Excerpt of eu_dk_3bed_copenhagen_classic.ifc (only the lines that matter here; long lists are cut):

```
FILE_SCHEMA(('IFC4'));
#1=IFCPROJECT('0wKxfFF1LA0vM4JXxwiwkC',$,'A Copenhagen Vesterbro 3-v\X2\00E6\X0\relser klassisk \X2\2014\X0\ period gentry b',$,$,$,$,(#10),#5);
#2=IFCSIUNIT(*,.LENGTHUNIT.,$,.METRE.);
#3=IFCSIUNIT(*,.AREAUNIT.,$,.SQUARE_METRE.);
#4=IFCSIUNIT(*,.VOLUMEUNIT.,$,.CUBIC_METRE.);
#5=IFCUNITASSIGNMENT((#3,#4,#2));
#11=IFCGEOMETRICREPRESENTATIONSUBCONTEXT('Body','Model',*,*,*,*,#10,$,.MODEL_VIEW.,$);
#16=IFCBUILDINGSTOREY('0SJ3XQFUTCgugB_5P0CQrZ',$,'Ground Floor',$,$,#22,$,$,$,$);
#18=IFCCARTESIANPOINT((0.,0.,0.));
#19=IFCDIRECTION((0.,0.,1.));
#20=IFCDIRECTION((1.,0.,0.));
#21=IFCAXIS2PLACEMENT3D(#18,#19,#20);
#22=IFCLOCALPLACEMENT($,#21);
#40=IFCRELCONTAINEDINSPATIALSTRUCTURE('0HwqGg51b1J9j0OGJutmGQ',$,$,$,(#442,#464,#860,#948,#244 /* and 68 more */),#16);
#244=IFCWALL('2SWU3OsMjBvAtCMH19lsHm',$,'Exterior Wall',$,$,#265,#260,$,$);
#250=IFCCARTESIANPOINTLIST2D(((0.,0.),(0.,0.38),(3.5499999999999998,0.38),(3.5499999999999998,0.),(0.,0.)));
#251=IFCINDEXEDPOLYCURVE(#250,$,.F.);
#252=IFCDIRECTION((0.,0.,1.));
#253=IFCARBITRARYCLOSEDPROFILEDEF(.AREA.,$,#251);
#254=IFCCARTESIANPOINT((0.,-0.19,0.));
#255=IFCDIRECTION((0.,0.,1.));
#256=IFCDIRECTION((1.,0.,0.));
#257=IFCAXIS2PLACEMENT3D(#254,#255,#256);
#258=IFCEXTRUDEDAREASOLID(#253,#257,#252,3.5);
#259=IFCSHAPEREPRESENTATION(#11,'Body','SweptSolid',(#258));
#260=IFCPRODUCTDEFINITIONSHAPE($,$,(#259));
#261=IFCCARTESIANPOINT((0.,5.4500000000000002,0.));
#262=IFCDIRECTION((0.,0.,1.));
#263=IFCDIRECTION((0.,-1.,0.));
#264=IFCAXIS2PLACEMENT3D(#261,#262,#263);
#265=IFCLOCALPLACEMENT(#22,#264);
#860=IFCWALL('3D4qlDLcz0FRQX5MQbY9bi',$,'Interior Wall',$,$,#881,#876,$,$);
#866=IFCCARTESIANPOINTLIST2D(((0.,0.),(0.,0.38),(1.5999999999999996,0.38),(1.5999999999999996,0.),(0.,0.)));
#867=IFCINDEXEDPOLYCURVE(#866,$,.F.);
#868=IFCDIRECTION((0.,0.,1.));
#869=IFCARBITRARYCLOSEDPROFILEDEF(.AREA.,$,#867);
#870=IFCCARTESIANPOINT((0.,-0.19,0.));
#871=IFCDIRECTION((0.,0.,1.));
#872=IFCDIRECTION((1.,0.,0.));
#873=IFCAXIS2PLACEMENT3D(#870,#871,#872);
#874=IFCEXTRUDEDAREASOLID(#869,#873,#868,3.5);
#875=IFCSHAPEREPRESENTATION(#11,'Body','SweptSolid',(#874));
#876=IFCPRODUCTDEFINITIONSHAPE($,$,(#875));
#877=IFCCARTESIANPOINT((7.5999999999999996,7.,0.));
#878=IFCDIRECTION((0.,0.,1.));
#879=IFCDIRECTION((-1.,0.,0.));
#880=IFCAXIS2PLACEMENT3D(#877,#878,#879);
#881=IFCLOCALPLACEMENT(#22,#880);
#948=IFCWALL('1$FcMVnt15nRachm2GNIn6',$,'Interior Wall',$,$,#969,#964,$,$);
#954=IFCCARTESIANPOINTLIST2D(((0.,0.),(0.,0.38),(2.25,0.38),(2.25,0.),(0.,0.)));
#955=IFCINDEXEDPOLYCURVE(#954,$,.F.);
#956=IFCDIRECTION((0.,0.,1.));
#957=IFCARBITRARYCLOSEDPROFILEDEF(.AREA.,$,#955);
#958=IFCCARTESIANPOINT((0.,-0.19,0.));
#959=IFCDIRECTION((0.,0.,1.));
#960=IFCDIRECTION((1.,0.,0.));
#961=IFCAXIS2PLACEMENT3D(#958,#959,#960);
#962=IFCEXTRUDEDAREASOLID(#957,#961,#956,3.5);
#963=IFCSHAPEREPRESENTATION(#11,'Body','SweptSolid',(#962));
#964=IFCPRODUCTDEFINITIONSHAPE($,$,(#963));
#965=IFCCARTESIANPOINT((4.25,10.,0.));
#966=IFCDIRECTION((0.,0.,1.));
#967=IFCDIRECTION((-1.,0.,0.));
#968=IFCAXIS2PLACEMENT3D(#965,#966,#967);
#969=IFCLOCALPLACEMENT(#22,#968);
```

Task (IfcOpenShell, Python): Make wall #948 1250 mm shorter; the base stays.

```python
import ifcopenshell
import ifcopenshell.geom
import ifcopenshell.util.representation
import ifcopenshell.util.shape
import ifcopenshell.util.unit

model = ifcopenshell.open("eu_dk_3bed_copenhagen_classic.ifc")
unit_scale = ifcopenshell.util.unit.calculate_unit_scale(model)
settings = ifcopenshell.geom.settings()


def volume(element):
    """Net volume in cubic metres, openings subtracted."""
    shape = ifcopenshell.geom.create_shape(settings, element)
    return ifcopenshell.util.shape.get_volume(shape.geometry)


wall = model.by_guid("1$FcMVnt15nRachm2GNIn6")
before = volume(wall)

body = ifcopenshell.util.representation.get_representation(wall, "Model", "Body")
solid = body.Items[0]
old_height = solid.Depth
solid.Depth -= 1.25 / unit_scale
after = volume(wall)

print(f"height {old_height:g} -> {solid.Depth:g}, volume {before:.3f} -> {after:.3f} m3")

model.write("eu_dk_3bed_copenhagen_classic_edited.ifc")
```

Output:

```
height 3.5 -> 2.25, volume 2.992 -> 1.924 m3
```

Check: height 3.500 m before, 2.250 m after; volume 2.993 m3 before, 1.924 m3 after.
